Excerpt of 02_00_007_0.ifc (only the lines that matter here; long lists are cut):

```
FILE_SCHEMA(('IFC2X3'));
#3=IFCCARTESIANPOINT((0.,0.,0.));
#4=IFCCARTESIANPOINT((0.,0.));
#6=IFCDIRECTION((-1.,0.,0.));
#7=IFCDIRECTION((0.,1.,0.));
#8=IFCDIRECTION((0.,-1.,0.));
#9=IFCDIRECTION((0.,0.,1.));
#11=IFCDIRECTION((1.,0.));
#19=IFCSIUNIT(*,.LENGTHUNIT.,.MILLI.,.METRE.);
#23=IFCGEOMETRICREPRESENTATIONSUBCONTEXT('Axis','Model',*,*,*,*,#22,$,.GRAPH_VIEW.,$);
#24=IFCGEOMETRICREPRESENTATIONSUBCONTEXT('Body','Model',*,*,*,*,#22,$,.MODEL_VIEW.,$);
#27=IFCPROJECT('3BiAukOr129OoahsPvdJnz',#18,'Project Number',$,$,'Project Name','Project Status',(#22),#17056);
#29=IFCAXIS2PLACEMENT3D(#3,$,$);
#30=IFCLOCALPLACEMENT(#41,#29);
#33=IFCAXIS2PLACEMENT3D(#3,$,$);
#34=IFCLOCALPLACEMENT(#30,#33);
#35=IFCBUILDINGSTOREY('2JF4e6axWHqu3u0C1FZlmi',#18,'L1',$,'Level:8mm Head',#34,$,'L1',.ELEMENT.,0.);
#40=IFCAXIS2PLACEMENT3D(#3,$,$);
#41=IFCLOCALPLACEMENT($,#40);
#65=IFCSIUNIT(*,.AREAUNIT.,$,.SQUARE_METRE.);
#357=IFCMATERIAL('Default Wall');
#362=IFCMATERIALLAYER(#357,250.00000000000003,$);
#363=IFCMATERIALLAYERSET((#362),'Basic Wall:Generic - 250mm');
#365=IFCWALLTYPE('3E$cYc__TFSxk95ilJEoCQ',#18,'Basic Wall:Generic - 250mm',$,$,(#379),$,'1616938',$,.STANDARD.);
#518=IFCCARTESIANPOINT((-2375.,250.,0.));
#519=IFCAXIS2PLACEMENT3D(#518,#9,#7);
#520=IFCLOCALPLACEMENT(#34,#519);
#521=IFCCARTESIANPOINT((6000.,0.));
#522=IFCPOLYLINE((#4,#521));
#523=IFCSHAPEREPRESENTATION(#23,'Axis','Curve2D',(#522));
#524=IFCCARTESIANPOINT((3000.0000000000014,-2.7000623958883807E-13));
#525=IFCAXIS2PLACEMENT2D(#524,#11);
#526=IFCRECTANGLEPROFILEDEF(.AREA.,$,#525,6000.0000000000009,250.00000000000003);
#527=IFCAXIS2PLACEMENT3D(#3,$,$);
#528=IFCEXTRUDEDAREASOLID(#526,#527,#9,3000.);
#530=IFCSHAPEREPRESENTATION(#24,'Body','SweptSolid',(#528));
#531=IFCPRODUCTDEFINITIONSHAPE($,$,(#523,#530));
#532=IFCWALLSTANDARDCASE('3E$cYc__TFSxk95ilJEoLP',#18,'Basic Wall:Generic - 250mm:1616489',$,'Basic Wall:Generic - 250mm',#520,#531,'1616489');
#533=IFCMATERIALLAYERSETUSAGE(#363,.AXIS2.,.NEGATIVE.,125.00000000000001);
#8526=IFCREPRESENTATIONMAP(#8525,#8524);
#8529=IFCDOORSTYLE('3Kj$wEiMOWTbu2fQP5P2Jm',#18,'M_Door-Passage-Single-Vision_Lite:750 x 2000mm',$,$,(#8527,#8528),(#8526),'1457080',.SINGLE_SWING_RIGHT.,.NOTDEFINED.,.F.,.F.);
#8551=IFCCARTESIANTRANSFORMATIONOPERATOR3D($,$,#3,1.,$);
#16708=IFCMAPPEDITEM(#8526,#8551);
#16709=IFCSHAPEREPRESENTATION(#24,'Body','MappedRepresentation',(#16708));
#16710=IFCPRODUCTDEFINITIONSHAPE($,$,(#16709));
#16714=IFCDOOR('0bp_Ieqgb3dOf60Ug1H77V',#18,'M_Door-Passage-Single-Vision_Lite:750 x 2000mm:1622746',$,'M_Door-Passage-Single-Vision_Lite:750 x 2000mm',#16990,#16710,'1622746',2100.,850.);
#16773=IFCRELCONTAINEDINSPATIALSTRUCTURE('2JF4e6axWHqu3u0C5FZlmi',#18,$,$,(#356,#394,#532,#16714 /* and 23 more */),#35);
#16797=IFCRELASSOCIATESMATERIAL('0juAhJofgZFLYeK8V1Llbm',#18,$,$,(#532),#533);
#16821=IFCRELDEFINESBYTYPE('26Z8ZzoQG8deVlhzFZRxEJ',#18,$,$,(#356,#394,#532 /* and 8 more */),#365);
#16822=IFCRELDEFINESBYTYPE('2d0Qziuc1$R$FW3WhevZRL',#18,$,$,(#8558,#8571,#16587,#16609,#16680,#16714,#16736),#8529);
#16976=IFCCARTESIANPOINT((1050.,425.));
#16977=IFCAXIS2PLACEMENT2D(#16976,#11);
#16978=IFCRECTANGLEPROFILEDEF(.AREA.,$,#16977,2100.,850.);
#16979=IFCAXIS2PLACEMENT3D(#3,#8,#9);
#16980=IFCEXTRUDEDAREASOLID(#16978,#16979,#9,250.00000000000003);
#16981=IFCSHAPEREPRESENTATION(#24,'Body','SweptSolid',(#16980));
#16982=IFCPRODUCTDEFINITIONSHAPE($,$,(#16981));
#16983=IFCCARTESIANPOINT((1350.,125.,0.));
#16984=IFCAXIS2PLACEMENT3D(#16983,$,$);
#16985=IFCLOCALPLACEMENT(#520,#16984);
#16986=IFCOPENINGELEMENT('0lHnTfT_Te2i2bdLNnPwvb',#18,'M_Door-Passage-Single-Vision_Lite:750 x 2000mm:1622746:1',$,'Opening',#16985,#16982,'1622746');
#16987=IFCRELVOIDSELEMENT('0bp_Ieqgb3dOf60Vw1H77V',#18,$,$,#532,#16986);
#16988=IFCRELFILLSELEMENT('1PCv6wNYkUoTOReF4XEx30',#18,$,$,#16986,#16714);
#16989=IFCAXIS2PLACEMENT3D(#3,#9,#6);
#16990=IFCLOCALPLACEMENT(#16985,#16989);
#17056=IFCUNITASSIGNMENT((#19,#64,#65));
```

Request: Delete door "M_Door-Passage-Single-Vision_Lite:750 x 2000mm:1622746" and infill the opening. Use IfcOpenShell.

```python
import ifcopenshell
import ifcopenshell.api.feature
import ifcopenshell.api.root
import ifcopenshell.geom
import ifcopenshell.util.shape

model = ifcopenshell.open("02_00_007_0.ifc")
settings = ifcopenshell.geom.settings()


def volume(element):
    """Net volume in cubic metres, openings subtracted."""
    shape = ifcopenshell.geom.create_shape(settings, element)
    return ifcopenshell.util.shape.get_volume(shape.geometry)


door = model.by_id(16714)
opening = door.FillsVoids[0].RelatingOpeningElement
wall = opening.VoidsElements[0].RelatingBuildingElement
before = volume(wall)

ifcopenshell.api.root.remove_product(model, product=door)
ifcopenshell.api.feature.remove_feature(model, feature=opening)

after = volume(wall)

print(f"wall volume {before:.3f} -> {after:.3f} m3")

model.write("02_00_007_0-out.ifc")
```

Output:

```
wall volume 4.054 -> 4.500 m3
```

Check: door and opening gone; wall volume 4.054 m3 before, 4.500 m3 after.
